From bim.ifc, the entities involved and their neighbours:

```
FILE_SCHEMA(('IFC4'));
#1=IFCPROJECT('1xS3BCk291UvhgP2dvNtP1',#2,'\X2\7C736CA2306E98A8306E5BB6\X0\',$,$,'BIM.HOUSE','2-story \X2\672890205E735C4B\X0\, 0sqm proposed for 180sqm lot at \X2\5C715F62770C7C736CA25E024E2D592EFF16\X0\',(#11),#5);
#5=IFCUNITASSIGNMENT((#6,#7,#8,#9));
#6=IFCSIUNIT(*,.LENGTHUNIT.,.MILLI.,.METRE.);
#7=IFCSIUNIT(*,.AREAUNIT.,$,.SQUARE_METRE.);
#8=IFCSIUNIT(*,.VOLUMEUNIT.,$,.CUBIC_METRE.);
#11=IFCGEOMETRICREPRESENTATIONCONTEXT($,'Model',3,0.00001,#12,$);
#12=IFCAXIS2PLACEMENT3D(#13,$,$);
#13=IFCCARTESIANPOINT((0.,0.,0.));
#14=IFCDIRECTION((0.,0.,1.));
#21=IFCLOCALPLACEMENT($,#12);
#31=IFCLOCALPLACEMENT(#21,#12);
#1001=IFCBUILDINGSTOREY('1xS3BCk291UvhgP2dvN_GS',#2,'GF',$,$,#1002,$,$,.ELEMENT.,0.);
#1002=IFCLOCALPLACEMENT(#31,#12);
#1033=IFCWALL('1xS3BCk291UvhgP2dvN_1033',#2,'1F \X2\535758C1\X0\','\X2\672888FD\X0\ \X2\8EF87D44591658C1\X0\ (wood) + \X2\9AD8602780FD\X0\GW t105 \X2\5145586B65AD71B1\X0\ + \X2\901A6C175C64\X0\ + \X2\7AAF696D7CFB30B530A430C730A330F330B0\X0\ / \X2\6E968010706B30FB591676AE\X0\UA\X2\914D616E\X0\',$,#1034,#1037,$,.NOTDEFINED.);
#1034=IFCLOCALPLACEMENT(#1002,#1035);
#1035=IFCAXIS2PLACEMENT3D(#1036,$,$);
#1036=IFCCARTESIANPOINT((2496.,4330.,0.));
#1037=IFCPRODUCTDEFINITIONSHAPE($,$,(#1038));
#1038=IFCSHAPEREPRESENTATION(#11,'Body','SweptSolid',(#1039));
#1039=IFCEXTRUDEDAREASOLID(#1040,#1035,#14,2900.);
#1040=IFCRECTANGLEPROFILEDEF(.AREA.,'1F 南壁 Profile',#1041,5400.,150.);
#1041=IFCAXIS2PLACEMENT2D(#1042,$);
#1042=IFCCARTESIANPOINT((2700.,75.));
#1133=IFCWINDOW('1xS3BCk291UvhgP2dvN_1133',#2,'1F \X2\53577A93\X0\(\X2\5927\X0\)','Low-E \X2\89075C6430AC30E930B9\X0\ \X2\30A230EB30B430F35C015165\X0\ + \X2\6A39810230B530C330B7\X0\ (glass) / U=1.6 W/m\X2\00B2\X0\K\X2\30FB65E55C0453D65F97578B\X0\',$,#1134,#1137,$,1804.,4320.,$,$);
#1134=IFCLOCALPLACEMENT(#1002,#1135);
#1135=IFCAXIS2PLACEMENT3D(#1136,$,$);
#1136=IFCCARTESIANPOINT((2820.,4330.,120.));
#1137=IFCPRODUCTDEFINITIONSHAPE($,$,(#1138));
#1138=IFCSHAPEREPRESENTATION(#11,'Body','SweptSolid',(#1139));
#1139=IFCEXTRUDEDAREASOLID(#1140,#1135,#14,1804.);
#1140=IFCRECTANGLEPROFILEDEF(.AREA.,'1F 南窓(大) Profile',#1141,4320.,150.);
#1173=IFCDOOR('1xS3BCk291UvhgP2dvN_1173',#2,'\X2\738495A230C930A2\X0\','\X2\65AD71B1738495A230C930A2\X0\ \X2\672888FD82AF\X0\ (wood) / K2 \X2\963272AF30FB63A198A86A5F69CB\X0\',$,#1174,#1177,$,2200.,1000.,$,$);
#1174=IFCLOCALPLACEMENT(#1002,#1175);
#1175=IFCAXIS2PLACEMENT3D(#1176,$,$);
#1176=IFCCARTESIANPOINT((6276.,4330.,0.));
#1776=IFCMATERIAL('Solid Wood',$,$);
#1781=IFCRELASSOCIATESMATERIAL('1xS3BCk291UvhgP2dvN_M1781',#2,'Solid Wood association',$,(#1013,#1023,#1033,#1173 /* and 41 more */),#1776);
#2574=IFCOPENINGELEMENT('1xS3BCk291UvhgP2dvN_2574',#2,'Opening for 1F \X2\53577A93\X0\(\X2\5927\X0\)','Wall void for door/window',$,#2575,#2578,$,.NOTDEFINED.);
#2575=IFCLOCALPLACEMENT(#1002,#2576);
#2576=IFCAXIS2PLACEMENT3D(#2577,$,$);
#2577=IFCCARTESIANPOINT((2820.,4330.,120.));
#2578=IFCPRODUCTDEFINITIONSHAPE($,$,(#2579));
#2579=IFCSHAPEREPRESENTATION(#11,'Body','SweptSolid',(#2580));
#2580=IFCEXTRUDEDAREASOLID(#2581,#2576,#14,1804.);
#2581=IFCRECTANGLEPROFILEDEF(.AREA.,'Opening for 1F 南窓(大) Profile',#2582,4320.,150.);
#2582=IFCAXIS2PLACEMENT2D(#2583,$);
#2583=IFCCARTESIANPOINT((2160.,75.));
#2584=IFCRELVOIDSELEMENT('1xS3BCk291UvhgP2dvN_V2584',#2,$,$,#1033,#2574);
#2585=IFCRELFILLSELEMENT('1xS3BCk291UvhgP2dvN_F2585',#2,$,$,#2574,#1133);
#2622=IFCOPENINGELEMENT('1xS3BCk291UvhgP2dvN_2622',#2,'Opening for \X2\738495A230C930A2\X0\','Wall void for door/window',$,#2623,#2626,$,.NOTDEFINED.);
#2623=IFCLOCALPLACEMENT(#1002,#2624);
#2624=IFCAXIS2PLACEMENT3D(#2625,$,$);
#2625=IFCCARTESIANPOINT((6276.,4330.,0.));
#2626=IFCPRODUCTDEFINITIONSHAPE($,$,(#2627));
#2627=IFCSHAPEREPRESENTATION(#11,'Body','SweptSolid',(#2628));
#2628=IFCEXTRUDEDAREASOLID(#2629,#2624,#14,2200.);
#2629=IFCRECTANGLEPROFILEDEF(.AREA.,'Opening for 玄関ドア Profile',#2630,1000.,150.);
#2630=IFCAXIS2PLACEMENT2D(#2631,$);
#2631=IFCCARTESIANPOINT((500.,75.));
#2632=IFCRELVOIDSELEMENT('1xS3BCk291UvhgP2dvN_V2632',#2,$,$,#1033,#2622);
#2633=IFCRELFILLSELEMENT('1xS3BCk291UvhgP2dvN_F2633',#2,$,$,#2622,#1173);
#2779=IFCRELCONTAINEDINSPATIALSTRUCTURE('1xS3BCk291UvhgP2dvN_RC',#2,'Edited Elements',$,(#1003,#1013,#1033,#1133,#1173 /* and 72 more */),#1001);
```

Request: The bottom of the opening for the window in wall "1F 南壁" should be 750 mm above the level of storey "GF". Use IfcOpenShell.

```python
import numpy as np
import ifcopenshell
import ifcopenshell.api.geometry
import ifcopenshell.geom
import ifcopenshell.util.element
import ifcopenshell.util.placement
import ifcopenshell.util.shape
import ifcopenshell.util.unit

model = ifcopenshell.open("bim.ifc")
unit_scale = ifcopenshell.util.unit.calculate_unit_scale(model)

window = model.by_guid("1xS3BCk291UvhgP2dvN_1133")
opening = window.FillsVoids[0].RelatingOpeningElement
storey = ifcopenshell.util.element.get_container(window, ifc_class="IfcBuildingStorey")
level = ifcopenshell.util.placement.get_local_placement(storey.ObjectPlacement)[2, 3]

# The opening's origin need not be at the sill, so measure its lowest point.
shape = ifcopenshell.geom.create_shape(ifcopenshell.geom.settings(), opening)
bottom = ifcopenshell.util.shape.get_shape_bottom_elevation(shape, shape.geometry) / unit_scale
dz = level + 0.75 / unit_scale - bottom

shift = np.array([0.0, 0.0, dz])
# The window is not placed relative to its opening, so move both.
for product in (opening, window):
    matrix = ifcopenshell.util.placement.get_local_placement(product.ObjectPlacement)
    matrix[:3, 3] += shift
    ifcopenshell.api.geometry.edit_object_placement(model, product=product, matrix=matrix, is_si=False)

print(f"moved by {dz * unit_scale:+.3f} m")

model.write("bim_updated.ifc")
```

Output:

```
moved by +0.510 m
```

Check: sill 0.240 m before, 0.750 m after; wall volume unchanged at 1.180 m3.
